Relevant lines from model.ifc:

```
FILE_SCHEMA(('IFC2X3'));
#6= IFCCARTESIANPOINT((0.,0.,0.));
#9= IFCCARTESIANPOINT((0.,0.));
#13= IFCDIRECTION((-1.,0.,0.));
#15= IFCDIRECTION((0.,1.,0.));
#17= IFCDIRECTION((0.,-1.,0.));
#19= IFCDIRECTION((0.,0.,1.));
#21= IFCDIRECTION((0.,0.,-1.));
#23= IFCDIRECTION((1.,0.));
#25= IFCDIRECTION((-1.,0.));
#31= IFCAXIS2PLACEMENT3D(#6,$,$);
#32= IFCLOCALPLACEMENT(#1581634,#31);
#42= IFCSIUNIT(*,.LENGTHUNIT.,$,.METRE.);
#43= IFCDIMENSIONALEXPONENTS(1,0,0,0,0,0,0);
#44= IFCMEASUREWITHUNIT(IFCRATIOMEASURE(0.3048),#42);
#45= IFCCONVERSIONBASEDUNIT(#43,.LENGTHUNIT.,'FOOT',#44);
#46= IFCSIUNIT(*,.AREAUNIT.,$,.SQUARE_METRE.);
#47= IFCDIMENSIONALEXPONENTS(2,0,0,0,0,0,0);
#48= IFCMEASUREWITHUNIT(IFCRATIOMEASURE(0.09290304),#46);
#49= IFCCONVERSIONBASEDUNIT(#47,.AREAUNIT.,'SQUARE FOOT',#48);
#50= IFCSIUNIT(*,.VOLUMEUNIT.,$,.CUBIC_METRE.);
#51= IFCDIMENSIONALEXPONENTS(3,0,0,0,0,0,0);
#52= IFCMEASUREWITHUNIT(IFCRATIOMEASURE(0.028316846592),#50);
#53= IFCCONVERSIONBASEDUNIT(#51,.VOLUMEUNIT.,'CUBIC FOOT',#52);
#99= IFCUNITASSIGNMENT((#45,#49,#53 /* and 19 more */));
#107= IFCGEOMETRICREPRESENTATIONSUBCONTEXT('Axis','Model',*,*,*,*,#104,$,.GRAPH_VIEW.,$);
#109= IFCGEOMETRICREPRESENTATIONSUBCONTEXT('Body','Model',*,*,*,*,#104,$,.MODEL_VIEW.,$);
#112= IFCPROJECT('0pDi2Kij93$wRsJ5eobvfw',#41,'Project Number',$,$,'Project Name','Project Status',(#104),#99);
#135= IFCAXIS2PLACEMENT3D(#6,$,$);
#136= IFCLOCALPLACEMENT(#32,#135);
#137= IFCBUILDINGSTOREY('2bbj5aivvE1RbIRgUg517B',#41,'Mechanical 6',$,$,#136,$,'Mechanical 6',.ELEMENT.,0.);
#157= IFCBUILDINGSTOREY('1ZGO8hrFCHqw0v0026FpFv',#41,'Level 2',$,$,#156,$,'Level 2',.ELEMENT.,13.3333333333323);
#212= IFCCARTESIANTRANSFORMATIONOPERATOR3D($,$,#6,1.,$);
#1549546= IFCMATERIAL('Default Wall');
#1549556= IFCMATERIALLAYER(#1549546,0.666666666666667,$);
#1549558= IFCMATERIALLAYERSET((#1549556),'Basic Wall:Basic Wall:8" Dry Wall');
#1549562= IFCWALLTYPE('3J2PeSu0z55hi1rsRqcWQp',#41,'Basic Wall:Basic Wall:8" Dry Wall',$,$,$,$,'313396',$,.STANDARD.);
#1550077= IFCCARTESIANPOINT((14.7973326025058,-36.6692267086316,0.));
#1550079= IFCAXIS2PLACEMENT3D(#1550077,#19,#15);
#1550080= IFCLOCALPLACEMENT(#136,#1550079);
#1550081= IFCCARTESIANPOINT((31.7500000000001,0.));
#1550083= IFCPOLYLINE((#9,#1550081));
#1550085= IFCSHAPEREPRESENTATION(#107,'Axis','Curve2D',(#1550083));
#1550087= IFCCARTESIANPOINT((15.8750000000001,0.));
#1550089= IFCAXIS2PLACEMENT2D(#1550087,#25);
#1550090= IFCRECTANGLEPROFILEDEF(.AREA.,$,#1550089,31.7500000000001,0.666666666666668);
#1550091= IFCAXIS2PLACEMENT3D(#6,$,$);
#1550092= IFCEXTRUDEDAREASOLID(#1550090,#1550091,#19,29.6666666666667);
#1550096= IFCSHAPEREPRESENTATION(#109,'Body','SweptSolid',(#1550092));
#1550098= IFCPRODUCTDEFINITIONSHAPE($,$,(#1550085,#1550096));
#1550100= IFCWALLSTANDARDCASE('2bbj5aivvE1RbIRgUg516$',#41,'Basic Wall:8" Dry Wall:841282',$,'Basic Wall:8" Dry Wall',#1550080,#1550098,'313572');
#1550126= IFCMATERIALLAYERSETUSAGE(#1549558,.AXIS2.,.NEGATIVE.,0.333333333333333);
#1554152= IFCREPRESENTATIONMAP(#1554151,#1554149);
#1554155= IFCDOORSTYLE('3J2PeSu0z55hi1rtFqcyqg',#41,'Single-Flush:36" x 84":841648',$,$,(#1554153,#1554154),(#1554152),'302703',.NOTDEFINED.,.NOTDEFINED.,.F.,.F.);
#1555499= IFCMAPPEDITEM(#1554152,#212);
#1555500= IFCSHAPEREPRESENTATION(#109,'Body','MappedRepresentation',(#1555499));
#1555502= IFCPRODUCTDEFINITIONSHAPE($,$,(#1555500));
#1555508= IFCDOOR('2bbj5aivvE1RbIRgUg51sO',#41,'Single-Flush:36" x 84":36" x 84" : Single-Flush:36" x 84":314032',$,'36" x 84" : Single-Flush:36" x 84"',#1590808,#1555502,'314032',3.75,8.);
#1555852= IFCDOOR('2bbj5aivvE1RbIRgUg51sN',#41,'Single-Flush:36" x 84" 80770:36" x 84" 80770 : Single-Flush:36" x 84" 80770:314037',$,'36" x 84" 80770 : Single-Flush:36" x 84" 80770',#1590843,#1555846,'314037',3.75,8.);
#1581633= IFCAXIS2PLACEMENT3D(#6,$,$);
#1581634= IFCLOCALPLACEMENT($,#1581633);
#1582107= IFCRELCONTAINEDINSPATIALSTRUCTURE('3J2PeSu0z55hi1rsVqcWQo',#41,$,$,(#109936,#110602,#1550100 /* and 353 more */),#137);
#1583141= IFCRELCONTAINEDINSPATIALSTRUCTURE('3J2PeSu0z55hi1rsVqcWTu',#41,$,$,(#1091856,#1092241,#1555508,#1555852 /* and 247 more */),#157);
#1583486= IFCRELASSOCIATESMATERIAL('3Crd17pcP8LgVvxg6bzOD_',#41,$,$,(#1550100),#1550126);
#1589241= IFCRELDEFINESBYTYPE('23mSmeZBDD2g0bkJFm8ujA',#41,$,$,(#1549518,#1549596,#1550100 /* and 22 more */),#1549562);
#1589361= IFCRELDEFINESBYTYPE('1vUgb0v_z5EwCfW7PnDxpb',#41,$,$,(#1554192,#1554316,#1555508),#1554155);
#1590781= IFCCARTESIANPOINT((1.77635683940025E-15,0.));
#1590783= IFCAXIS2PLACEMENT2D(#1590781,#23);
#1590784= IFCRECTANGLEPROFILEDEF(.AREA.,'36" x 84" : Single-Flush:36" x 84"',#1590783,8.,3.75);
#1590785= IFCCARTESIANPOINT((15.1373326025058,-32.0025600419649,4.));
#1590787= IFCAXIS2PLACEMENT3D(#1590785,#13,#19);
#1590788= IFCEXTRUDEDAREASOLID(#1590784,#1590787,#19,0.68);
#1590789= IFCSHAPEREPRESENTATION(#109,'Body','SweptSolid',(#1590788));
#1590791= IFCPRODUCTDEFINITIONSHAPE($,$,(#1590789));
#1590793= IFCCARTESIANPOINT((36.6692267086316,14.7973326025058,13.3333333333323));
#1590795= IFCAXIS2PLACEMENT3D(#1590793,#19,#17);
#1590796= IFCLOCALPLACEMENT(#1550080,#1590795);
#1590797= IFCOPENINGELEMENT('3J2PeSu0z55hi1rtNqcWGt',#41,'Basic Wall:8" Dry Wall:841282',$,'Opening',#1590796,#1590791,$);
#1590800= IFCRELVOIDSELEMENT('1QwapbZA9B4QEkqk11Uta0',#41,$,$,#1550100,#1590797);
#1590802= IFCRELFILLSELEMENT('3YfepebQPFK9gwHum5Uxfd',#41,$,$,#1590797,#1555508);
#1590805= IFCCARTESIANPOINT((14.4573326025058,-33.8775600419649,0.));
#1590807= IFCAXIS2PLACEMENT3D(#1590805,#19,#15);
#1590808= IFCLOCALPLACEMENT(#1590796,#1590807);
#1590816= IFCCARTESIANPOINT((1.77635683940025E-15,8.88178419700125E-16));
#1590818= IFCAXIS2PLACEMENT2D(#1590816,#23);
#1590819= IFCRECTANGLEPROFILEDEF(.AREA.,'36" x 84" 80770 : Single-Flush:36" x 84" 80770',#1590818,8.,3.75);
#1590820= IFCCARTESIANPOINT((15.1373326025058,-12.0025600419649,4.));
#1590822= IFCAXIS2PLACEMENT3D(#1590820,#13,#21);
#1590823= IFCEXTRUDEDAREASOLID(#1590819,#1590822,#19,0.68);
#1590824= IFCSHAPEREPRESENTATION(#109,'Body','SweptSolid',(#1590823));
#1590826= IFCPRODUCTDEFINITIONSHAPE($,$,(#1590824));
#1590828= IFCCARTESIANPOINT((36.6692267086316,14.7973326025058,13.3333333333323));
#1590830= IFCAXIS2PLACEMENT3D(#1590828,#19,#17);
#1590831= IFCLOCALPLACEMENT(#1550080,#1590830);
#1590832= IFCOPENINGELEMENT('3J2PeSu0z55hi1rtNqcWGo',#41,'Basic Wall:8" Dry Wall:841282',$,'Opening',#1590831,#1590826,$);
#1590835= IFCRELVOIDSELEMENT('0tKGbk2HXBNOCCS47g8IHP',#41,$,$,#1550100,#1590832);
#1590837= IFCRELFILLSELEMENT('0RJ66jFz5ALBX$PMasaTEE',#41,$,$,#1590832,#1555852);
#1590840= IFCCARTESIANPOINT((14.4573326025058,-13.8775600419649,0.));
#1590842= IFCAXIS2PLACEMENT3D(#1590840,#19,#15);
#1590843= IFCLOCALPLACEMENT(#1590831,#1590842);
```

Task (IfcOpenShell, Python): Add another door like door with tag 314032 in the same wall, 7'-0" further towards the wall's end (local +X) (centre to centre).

```python
import ifcopenshell
import ifcopenshell.api.feature
import ifcopenshell.api.geometry
import ifcopenshell.api.root
import ifcopenshell.geom
import ifcopenshell.util.element
import ifcopenshell.util.placement
import ifcopenshell.util.shape
import ifcopenshell.util.unit

model = ifcopenshell.open("model.ifc")
unit_scale = ifcopenshell.util.unit.calculate_unit_scale(model)
settings = ifcopenshell.geom.settings()


def volume(element):
    """Net volume in cubic metres, openings subtracted."""
    shape = ifcopenshell.geom.create_shape(settings, element)
    return ifcopenshell.util.shape.get_volume(shape.geometry)


def reuse_history(source, copy):
    """copy_class also copies each property set's owner history, people and application; keep the originals."""
    for rel in copy.IsDefinedBy:
        if rel.is_a("IfcRelDefinesByProperties") and (history := rel.RelatingPropertyDefinition.OwnerHistory):
            rel.RelatingPropertyDefinition.OwnerHistory = source.OwnerHistory
            ifcopenshell.util.element.remove_deep2(model, history)


door = model.by_id(1555508)
opening = door.FillsVoids[0].RelatingOpeningElement
wall = opening.VoidsElements[0].RelatingBuildingElement
before = volume(wall)
shift = ifcopenshell.util.placement.get_local_placement(wall.ObjectPlacement)[:3, 0] * 84 * 0.0254 / unit_scale

# copy_class copies the void relationship, type, container and properties, but no geometry.
new_opening = ifcopenshell.api.root.copy_class(model, product=opening)
new_opening.Representation = ifcopenshell.util.element.copy_deep(
    model, opening.Representation, exclude=["IfcGeometricRepresentationContext", "IfcRepresentationMap"]
)
new_opening.Name = 'Basic Wall:8" Dry Wall'
new_door = ifcopenshell.api.root.copy_class(model, product=door)
new_door.Representation = ifcopenshell.util.element.copy_deep(
    model, door.Representation, exclude=["IfcGeometricRepresentationContext", "IfcRepresentationMap"]
)
new_door.Name = 'Single-Flush:36" x 84":36" x 84" : Single-Flush:36" x 84"'
new_door.Tag = None
reuse_history(door, new_door)
fills = ifcopenshell.api.feature.add_filling(model, opening=new_opening, element=new_door)
fills.OwnerHistory = new_door.OwnerHistory  # required in IFC2X3

for old, new in ((opening, new_opening), (door, new_door)):
    matrix = ifcopenshell.util.placement.get_local_placement(old.ObjectPlacement)
    matrix[:3, 3] += shift
    ifcopenshell.api.geometry.edit_object_placement(model, product=new, matrix=matrix, is_si=False)

after = volume(wall)

print(f"wall volume {before:.3f} -> {after:.3f} m3")

model.write("model-out.ifc")
```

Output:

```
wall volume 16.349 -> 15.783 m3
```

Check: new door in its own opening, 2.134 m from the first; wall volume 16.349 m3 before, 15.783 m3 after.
